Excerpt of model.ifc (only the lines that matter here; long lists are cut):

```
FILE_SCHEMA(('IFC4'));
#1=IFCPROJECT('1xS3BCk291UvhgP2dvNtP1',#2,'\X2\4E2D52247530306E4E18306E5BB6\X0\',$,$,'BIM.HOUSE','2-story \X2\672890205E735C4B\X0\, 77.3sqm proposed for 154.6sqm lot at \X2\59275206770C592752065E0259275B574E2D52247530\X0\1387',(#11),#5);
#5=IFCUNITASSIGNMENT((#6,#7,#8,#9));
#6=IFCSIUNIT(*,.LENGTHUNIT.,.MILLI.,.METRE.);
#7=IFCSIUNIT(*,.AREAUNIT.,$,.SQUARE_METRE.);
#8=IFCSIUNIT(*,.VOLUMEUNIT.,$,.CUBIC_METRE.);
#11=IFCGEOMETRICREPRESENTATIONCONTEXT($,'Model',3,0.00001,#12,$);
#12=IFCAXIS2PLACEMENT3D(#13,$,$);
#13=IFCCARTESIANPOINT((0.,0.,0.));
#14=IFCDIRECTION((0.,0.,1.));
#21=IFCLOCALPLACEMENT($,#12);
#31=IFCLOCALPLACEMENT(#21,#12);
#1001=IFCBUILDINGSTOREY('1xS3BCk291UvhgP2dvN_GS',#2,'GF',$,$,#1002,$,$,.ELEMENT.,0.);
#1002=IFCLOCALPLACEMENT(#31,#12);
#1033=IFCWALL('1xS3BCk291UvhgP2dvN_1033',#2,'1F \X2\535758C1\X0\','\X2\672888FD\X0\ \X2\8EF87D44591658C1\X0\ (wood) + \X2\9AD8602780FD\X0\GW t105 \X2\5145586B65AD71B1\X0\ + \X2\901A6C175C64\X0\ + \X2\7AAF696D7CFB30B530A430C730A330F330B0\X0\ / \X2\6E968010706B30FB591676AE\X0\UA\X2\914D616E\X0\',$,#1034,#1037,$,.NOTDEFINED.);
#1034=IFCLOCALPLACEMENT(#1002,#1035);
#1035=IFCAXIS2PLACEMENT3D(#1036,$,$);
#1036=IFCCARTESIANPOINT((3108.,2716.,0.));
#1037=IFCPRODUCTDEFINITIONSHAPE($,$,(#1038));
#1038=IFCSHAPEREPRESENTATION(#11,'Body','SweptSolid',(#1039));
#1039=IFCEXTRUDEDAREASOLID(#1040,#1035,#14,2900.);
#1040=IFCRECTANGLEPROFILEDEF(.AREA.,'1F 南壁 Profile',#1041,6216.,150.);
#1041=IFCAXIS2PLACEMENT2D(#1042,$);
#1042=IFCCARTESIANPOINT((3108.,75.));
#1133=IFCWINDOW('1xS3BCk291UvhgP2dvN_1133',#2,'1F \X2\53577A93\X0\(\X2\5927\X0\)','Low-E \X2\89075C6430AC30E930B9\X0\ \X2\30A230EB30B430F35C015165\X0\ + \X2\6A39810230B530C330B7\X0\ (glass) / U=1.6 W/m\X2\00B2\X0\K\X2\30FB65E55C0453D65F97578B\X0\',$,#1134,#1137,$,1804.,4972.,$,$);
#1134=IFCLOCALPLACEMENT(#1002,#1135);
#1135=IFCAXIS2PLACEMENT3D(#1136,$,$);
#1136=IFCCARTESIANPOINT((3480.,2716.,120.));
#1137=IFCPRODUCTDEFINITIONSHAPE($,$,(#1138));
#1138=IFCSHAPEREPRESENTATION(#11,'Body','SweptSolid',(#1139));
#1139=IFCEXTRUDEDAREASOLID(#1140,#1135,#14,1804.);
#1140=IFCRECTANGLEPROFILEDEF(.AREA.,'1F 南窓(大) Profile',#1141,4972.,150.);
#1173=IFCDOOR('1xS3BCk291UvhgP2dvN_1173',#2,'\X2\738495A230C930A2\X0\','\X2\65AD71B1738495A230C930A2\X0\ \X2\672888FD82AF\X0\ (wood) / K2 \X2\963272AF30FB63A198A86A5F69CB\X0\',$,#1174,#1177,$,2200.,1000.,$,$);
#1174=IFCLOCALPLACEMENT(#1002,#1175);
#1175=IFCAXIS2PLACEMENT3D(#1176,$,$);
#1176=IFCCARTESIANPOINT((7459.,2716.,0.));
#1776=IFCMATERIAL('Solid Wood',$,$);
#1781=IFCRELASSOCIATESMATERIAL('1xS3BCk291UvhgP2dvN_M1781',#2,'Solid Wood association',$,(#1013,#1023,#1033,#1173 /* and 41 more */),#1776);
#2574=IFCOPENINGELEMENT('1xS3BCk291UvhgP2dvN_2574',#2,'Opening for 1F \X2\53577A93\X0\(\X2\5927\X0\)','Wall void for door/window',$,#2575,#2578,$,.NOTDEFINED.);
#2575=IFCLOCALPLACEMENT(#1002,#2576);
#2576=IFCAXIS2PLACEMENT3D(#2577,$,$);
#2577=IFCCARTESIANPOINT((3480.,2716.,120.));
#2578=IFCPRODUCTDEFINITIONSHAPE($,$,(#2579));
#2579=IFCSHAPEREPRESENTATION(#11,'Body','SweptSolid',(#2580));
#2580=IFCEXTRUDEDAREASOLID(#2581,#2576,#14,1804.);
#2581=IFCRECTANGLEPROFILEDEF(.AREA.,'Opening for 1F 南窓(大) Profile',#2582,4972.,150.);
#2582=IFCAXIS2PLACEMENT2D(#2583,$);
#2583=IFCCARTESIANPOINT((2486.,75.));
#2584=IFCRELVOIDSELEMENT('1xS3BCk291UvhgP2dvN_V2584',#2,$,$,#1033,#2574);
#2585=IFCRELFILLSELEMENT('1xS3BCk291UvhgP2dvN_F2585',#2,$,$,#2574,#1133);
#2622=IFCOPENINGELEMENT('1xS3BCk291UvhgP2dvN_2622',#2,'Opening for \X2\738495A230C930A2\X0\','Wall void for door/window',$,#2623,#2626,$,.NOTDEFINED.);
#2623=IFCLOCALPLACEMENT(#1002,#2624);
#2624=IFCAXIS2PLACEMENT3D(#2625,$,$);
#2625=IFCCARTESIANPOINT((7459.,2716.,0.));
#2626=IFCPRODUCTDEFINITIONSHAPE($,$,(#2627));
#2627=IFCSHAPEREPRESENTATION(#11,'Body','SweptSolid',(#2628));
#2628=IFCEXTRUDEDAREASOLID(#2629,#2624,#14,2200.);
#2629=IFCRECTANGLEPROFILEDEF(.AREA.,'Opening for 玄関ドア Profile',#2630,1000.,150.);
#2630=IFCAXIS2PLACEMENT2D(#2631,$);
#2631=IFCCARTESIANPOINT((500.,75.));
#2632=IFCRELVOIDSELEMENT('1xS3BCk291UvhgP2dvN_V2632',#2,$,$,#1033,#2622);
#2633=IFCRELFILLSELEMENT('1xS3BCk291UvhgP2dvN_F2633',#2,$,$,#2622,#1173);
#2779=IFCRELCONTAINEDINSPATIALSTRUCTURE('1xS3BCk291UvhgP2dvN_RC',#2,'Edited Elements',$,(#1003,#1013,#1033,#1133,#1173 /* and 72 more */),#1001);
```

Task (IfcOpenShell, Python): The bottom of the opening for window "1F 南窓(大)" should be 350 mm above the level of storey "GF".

```python
import numpy as np
import ifcopenshell
import ifcopenshell.api.geometry
import ifcopenshell.geom
import ifcopenshell.util.element
import ifcopenshell.util.placement
import ifcopenshell.util.shape
import ifcopenshell.util.unit

model = ifcopenshell.open("model.ifc")
unit_scale = ifcopenshell.util.unit.calculate_unit_scale(model)

window = model.by_guid("1xS3BCk291UvhgP2dvN_1133")
opening = window.FillsVoids[0].RelatingOpeningElement
storey = ifcopenshell.util.element.get_container(window, ifc_class="IfcBuildingStorey")
level = ifcopenshell.util.placement.get_local_placement(storey.ObjectPlacement)[2, 3]

# The opening's origin need not be at the sill, so measure its lowest point.
shape = ifcopenshell.geom.create_shape(ifcopenshell.geom.settings(), opening)
bottom = ifcopenshell.util.shape.get_shape_bottom_elevation(shape, shape.geometry) / unit_scale
dz = level + 350.0 - bottom

shift = np.array([0.0, 0.0, dz])
# The window is not placed relative to its opening, so move both.
for product in (opening, window):
    matrix = ifcopenshell.util.placement.get_local_placement(product.ObjectPlacement)
    matrix[:3, 3] += shift
    ifcopenshell.api.geometry.edit_object_placement(model, product=product, matrix=matrix, is_si=False)

print(f"moved by {dz * unit_scale:+.3f} m")

model.write("model_edited.ifc")
```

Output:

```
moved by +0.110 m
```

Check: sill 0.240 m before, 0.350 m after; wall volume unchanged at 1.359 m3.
